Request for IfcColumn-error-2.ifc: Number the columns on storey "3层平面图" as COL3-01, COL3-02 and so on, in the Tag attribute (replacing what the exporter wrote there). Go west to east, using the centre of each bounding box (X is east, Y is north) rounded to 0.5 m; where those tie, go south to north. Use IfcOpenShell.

First a look at what the model holds.

```python
import ifcopenshell
import ifcopenshell.util.element
import ifcopenshell.util.placement

model = ifcopenshell.open("IfcColumn-error-2.ifc")
print(model.schema)
storey = next(s for s in model.by_type("IfcBuildingStorey") if s.Name == "3层平面图")
columns = [e for e in ifcopenshell.util.element.get_decomposition(storey) if e.is_a("IfcColumn")]
for e in sorted(columns, key=lambda e: e.id()):
    origin = ifcopenshell.util.placement.get_local_placement(e.ObjectPlacement)[:3, 3]
    print(e.id(), e.Tag, e.Name, origin.round(2) + 0.0, sep=" | ")
```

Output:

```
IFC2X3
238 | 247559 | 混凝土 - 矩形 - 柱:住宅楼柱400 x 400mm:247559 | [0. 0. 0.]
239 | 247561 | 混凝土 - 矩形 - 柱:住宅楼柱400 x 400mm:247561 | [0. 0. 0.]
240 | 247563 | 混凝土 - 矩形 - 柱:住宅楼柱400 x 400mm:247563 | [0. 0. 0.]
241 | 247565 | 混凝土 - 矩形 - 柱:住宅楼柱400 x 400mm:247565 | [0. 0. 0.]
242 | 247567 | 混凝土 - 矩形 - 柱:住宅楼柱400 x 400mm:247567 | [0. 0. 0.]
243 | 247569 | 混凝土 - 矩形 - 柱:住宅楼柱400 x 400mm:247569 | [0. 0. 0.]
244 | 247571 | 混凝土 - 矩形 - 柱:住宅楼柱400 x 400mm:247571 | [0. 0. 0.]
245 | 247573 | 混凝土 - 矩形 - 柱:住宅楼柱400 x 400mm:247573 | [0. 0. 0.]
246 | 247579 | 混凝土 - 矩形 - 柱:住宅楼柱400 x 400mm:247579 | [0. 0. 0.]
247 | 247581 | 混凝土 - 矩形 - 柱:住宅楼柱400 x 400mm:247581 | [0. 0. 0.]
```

```python
import ifcopenshell
import ifcopenshell.geom
import ifcopenshell.util.element
import ifcopenshell.util.shape

model = ifcopenshell.open("IfcColumn-error-2.ifc")
settings = ifcopenshell.geom.settings()
settings.set("use-world-coords", True)


def centre(element):
    shape = ifcopenshell.geom.create_shape(settings, element)
    return ifcopenshell.util.shape.get_bbox_centroid(shape.geometry)


storey = next(s for s in model.by_type("IfcBuildingStorey") if s.Name == "3层平面图")
columns = [e for e in ifcopenshell.util.element.get_decomposition(storey) if e.is_a("IfcColumn")]

# Insertion points can sit at a corner or the storey origin, so sort by the geometry (in metres).
centres = {e: centre(e) for e in columns}
columns.sort(key=lambda e: (round(centres[e][0] / 0.5), centres[e][1]))

for i, e in enumerate(columns, start=1):
    number = f"COL3-{i:02d}"
    e.Tag = number
    print(e.id(), number)

model.write("IfcColumn-error-2_v2.ifc")
```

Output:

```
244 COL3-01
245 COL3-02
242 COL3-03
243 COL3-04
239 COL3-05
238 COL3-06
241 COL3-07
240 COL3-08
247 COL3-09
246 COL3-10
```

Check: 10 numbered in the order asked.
